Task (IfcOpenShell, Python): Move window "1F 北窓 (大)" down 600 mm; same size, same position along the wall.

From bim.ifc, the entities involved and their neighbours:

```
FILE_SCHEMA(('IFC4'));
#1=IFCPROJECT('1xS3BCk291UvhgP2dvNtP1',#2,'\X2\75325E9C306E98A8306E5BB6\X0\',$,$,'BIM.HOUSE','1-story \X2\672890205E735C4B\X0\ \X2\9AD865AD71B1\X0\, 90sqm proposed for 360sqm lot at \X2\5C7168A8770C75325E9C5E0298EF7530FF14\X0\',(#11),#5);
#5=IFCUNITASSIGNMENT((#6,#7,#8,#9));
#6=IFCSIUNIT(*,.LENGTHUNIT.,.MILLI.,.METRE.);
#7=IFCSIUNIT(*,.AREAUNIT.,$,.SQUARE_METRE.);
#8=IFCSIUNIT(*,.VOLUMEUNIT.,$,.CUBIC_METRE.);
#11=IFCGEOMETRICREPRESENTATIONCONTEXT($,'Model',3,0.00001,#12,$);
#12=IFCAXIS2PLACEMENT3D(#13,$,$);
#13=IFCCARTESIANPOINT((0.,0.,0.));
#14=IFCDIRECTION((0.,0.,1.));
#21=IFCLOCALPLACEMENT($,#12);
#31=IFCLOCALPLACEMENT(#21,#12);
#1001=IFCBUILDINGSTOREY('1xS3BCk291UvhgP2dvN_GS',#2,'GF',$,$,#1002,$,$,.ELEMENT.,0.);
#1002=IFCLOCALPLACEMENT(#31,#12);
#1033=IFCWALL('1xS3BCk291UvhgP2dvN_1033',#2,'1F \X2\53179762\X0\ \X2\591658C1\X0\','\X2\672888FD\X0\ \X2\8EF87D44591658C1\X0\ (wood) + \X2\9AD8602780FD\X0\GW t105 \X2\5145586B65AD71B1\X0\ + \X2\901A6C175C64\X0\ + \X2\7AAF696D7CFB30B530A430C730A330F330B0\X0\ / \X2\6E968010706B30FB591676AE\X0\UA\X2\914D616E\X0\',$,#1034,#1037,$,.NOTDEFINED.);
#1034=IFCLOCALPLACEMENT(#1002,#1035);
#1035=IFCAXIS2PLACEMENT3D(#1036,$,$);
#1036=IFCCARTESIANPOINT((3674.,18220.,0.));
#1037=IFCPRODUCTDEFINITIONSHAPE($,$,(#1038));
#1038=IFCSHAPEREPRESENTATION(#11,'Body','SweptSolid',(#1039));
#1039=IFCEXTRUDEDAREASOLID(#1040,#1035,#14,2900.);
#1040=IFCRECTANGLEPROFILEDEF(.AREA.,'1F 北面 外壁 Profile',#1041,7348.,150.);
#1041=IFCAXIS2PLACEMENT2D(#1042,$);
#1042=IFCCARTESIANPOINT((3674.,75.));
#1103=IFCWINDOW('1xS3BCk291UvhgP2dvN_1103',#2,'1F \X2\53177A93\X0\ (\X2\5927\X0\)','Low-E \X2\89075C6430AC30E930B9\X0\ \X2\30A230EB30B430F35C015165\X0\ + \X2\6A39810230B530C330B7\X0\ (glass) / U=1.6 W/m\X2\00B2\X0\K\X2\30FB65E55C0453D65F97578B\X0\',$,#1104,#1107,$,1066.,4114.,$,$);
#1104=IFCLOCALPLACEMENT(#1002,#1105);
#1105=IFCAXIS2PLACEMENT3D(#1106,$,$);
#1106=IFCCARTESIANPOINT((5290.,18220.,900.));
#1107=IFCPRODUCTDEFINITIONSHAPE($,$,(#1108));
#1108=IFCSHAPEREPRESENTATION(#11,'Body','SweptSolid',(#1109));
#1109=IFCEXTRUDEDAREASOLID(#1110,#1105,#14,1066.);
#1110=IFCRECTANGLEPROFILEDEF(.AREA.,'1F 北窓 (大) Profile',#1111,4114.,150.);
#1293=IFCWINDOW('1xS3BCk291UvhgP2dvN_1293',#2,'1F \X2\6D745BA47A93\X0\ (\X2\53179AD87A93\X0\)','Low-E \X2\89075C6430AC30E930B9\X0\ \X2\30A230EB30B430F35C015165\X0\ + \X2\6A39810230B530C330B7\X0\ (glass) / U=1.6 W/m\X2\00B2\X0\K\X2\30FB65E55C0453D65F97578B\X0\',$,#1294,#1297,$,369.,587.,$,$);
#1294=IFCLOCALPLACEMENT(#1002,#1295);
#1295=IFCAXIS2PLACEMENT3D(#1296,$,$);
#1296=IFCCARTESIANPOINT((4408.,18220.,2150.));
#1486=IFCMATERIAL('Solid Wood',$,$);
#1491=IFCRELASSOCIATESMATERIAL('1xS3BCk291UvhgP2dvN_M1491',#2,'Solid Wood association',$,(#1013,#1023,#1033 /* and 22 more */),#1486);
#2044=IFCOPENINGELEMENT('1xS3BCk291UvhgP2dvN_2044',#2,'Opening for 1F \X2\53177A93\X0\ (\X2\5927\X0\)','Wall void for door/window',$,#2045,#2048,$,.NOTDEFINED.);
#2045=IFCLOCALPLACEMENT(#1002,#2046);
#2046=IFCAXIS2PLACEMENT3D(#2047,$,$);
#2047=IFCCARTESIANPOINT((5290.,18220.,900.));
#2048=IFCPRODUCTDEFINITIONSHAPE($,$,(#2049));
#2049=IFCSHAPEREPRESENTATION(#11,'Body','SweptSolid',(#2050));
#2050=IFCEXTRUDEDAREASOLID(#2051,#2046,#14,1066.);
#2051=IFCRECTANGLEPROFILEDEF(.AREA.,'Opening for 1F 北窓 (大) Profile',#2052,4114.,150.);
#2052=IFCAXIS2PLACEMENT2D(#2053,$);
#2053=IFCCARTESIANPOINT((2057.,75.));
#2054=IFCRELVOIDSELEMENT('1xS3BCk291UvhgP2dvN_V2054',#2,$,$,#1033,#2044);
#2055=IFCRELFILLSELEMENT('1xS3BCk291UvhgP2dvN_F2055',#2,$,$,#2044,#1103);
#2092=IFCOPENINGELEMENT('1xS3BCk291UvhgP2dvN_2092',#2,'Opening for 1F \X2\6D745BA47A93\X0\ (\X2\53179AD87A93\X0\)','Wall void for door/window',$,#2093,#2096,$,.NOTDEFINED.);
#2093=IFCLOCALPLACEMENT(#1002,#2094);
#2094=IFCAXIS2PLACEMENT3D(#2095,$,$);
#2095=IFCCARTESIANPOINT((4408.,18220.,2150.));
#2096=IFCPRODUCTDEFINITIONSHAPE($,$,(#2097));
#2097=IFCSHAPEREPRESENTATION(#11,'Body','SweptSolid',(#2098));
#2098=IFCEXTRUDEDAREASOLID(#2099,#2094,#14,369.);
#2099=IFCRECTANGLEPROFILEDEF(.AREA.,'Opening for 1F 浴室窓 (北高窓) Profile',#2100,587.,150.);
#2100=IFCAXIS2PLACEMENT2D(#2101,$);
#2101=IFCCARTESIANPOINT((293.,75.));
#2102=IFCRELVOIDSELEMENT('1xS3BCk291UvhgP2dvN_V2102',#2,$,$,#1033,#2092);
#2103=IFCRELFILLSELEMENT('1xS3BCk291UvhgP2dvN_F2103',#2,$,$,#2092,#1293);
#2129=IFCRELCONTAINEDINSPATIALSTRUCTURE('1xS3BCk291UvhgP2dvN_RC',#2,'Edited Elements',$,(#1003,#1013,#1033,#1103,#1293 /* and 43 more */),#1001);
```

```python
import numpy as np
import ifcopenshell
import ifcopenshell.api.geometry
import ifcopenshell.util.placement
import ifcopenshell.util.unit

model = ifcopenshell.open("bim.ifc")
unit_scale = ifcopenshell.util.unit.calculate_unit_scale(model)

window = model.by_id(1103)
opening = window.FillsVoids[0].RelatingOpeningElement
dz = -0.6 / unit_scale

shift = np.array([0.0, 0.0, dz])
# The window is not placed relative to its opening, so move both.
for product in (opening, window):
    matrix = ifcopenshell.util.placement.get_local_placement(product.ObjectPlacement)
    matrix[:3, 3] += shift
    ifcopenshell.api.geometry.edit_object_placement(model, product=product, matrix=matrix, is_si=False)

print(f"moved by {dz * unit_scale:+.3f} m")

model.write("bim-out.ifc")
```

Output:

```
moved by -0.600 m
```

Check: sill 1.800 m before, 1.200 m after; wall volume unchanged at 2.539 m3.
